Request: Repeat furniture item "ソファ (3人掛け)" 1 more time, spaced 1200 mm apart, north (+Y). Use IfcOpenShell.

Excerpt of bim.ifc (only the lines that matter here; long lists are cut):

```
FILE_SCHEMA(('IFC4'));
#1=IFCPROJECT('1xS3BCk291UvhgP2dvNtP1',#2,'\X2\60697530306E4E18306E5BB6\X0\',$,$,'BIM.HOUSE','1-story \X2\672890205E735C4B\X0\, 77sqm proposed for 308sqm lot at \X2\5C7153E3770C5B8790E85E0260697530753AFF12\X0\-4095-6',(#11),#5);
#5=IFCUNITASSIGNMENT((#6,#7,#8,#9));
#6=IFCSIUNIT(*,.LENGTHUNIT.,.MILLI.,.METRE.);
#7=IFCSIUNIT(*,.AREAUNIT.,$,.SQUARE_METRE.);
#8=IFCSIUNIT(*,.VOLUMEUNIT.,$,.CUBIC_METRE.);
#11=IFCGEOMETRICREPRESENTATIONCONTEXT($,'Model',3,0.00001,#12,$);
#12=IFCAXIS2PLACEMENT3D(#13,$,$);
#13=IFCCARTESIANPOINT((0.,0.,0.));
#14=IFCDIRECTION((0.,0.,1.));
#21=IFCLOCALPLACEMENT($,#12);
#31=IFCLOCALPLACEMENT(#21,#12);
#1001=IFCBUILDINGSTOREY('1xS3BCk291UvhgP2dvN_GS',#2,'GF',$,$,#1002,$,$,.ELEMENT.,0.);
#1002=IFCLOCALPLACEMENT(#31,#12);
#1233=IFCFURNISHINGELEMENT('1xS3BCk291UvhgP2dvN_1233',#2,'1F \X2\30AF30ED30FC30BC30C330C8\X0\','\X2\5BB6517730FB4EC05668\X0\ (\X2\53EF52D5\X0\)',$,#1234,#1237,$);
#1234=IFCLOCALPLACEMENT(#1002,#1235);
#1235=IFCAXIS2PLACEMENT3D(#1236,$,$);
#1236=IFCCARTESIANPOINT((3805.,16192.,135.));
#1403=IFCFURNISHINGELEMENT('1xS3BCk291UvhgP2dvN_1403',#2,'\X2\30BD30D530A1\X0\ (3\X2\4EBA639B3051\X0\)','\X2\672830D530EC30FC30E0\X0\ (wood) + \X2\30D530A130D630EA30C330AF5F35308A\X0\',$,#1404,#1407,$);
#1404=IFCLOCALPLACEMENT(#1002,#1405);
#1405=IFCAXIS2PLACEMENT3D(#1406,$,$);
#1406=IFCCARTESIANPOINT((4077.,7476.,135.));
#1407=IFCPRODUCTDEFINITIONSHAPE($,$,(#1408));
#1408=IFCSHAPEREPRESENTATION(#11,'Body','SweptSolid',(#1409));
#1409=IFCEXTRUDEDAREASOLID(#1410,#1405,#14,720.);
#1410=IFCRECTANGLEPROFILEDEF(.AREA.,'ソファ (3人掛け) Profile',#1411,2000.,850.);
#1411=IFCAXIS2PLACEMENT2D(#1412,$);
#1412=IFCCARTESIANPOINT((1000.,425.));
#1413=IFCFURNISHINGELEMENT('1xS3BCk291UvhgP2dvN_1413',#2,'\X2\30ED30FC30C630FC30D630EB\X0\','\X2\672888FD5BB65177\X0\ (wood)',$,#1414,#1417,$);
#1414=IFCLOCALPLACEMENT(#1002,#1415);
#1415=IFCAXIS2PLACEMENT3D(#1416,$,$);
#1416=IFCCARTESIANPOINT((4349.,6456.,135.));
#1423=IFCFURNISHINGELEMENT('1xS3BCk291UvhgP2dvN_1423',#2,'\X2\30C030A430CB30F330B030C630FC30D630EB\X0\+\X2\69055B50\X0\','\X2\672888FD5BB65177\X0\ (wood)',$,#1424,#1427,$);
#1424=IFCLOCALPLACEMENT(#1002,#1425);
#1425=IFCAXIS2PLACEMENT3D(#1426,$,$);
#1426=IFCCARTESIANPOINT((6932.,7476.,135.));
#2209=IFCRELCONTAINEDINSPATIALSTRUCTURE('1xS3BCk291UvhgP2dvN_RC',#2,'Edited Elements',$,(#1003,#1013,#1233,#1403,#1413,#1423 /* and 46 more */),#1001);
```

```python
import numpy as np
import ifcopenshell
import ifcopenshell.api.geometry
import ifcopenshell.api.root
import ifcopenshell.util.element
import ifcopenshell.util.placement
import ifcopenshell.util.unit

model = ifcopenshell.open("bim.ifc")
unit_scale = ifcopenshell.util.unit.calculate_unit_scale(model)


def reuse_history(source, copy):
    """copy_class also copies each property set's owner history, people and application; keep the originals."""
    for rel in copy.IsDefinedBy:
        if rel.is_a("IfcRelDefinesByProperties") and (history := rel.RelatingPropertyDefinition.OwnerHistory):
            rel.RelatingPropertyDefinition.OwnerHistory = source.OwnerHistory
            ifcopenshell.util.element.remove_deep2(model, history)


source = model.by_id(1403)
base = ifcopenshell.util.placement.get_local_placement(source.ObjectPlacement)
step = np.array([0.0, 1.0, 0.0]) * 1.2 / unit_scale

for i in range(1, 2):
    copy = ifcopenshell.api.root.copy_class(model, product=source)
    copy.Representation = ifcopenshell.util.element.copy_deep(
        model, source.Representation, exclude=["IfcGeometricRepresentationContext", "IfcRepresentationMap"]
    )
    reuse_history(source, copy)
    matrix = base.copy()
    matrix[:3, 3] += i * step
    print("added at", matrix[:3, 3].round(3) + 0.0)
    ifcopenshell.api.geometry.edit_object_placement(model, product=copy, matrix=matrix, is_si=False)

model.write("bim_rev.ifc")
```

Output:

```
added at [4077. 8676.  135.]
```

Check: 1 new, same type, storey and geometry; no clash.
